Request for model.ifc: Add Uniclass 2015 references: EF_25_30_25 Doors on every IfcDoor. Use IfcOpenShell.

First a look at what the model holds.

```python
import ifcopenshell

model = ifcopenshell.open("model.ifc")
print(model.schema)
print("classifications:", [c.Name for c in model.by_type("IfcClassification")])
for ifc_class in ("IfcDoor", "IfcRoof", "IfcStair", "IfcWall", "IfcWindow"):
    print(ifc_class, len(model.by_type(ifc_class)))
```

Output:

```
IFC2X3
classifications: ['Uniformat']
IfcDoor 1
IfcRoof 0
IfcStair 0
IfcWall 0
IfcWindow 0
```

```python
import ifcopenshell
import ifcopenshell.api.classification

model = ifcopenshell.open("model.ifc")

# IFC2X3 requires Source and Edition and has no link from the project to the system.
system = model.create_entity("IfcClassification", Source="NBS", Edition="2015", Name="Uniclass 2015")

codes = {
    "IfcDoor": ("EF_25_30_25", "Doors"),
}
for ifc_class, (code, name) in codes.items():
    products = model.by_type(ifc_class)
    ifcopenshell.api.classification.add_reference(
        model, products=products, classification=system, identification=code, name=name
    )
    print(code, len(products))

model.write("model_v2.ifc")
```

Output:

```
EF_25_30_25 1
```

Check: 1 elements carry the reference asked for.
